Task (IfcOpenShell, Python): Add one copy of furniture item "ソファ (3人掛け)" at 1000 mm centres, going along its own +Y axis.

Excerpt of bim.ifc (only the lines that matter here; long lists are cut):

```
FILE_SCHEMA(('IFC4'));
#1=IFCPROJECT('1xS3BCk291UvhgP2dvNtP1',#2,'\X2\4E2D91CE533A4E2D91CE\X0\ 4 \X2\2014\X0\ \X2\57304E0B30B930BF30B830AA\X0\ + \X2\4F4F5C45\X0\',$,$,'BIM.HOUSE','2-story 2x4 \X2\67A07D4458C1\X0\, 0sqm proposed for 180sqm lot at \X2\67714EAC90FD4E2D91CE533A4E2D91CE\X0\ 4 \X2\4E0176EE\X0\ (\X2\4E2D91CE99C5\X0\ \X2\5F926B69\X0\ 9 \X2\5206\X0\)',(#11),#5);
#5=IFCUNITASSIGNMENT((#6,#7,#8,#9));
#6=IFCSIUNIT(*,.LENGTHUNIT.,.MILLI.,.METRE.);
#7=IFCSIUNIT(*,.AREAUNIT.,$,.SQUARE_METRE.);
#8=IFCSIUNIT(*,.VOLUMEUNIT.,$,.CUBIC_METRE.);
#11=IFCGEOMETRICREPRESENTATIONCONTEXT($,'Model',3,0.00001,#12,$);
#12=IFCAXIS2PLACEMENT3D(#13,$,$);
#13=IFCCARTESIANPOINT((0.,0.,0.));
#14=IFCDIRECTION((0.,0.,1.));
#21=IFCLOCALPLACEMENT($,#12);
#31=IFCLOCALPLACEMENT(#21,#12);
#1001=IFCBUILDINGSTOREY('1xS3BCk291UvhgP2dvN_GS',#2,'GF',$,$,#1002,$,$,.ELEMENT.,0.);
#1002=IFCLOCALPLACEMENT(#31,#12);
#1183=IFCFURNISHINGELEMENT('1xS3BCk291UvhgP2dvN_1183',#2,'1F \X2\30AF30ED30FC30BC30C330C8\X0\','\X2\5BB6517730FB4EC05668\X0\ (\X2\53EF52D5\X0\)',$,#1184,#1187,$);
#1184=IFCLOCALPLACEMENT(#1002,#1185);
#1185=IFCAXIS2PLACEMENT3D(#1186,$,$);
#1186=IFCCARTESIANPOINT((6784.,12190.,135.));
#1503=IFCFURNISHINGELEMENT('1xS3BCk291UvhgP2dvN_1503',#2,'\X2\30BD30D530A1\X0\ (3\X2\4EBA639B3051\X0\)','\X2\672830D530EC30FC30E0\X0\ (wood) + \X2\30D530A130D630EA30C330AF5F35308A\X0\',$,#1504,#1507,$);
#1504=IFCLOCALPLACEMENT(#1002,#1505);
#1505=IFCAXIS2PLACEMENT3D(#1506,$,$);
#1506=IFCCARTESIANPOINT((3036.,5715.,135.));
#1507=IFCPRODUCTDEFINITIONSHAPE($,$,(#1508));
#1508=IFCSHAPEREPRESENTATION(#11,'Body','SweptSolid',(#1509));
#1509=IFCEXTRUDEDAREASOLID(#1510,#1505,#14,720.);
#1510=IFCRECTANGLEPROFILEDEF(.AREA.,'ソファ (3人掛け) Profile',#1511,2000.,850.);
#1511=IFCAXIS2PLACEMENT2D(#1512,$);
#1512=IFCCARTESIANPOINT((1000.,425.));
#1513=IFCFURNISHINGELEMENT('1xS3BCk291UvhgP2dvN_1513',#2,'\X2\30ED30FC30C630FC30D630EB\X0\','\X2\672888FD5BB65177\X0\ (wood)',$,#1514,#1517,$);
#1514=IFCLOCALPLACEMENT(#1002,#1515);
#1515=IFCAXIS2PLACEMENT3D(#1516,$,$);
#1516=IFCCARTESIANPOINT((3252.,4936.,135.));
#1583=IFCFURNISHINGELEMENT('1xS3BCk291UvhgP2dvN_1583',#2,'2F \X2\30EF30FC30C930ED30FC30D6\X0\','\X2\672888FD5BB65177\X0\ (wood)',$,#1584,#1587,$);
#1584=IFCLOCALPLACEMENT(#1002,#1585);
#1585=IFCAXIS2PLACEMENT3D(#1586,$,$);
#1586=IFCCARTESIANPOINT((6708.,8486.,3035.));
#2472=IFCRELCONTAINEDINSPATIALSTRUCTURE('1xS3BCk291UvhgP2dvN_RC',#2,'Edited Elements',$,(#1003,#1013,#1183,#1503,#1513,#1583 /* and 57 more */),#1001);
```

```python
import ifcopenshell
import ifcopenshell.api.geometry
import ifcopenshell.api.root
import ifcopenshell.util.element
import ifcopenshell.util.placement

model = ifcopenshell.open("bim.ifc")


def reuse_history(source, copy):
    """copy_class also copies each property set's owner history, people and application; keep the originals."""
    for rel in copy.IsDefinedBy:
        if rel.is_a("IfcRelDefinesByProperties") and (history := rel.RelatingPropertyDefinition.OwnerHistory):
            rel.RelatingPropertyDefinition.OwnerHistory = source.OwnerHistory
            ifcopenshell.util.element.remove_deep2(model, history)


source = model.by_guid("1xS3BCk291UvhgP2dvN_1503")
base = ifcopenshell.util.placement.get_local_placement(source.ObjectPlacement)
step = base[:3, 1] * 1000.0

for i in range(1, 2):
    copy = ifcopenshell.api.root.copy_class(model, product=source)
    copy.Representation = ifcopenshell.util.element.copy_deep(
        model, source.Representation, exclude=["IfcGeometricRepresentationContext", "IfcRepresentationMap"]
    )
    reuse_history(source, copy)
    matrix = base.copy()
    matrix[:3, 3] += i * step
    print("added at", matrix[:3, 3].round(3) + 0.0)
    ifcopenshell.api.geometry.edit_object_placement(model, product=copy, matrix=matrix, is_si=False)

model.write("bim-out.ifc")
```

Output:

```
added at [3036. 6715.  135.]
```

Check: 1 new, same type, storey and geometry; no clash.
